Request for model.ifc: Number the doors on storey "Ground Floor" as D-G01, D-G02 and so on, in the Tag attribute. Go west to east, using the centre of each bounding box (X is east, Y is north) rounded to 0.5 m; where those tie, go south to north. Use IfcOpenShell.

First a look at what the model holds.

```python
import ifcopenshell
import ifcopenshell.util.element
import ifcopenshell.util.placement

model = ifcopenshell.open("model.ifc")
print(model.schema)
storey = next(s for s in model.by_type("IfcBuildingStorey") if s.Name == "Ground Floor")
doors = [e for e in ifcopenshell.util.element.get_decomposition(storey) if e.is_a("IfcDoor")]
for e in sorted(doors, key=lambda e: e.id()):
    origin = ifcopenshell.util.placement.get_local_placement(e.ObjectPlacement)[:3, 3]
    print(e.id(), e.Tag, e.Name, origin.round(2) + 0.0, sep=" | ")
```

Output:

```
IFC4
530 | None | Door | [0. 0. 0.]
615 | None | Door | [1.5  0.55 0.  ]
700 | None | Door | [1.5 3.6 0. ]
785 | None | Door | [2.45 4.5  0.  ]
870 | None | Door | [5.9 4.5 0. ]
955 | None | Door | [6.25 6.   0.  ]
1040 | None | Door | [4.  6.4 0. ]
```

```python
import ifcopenshell
import ifcopenshell.geom
import ifcopenshell.util.element
import ifcopenshell.util.shape

model = ifcopenshell.open("model.ifc")
settings = ifcopenshell.geom.settings()
settings.set("use-world-coords", True)


def centre(element):
    shape = ifcopenshell.geom.create_shape(settings, element)
    return ifcopenshell.util.shape.get_bbox_centroid(shape.geometry)


storey = next(s for s in model.by_type("IfcBuildingStorey") if s.Name == "Ground Floor")
doors = [e for e in ifcopenshell.util.element.get_decomposition(storey) if e.is_a("IfcDoor")]

# Insertion points can sit at a corner or the storey origin, so sort by the geometry (in metres).
centres = {e: centre(e) for e in doors}
doors.sort(key=lambda e: (round(centres[e][0] / 0.5), centres[e][1]))

for i, e in enumerate(doors, start=1):
    number = f"D-G{i:02d}"
    e.Tag = number
    print(e.id(), number)

model.write("model_v2.ifc")
```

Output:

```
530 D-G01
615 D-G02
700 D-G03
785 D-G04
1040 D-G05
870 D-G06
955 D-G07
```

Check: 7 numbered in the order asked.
